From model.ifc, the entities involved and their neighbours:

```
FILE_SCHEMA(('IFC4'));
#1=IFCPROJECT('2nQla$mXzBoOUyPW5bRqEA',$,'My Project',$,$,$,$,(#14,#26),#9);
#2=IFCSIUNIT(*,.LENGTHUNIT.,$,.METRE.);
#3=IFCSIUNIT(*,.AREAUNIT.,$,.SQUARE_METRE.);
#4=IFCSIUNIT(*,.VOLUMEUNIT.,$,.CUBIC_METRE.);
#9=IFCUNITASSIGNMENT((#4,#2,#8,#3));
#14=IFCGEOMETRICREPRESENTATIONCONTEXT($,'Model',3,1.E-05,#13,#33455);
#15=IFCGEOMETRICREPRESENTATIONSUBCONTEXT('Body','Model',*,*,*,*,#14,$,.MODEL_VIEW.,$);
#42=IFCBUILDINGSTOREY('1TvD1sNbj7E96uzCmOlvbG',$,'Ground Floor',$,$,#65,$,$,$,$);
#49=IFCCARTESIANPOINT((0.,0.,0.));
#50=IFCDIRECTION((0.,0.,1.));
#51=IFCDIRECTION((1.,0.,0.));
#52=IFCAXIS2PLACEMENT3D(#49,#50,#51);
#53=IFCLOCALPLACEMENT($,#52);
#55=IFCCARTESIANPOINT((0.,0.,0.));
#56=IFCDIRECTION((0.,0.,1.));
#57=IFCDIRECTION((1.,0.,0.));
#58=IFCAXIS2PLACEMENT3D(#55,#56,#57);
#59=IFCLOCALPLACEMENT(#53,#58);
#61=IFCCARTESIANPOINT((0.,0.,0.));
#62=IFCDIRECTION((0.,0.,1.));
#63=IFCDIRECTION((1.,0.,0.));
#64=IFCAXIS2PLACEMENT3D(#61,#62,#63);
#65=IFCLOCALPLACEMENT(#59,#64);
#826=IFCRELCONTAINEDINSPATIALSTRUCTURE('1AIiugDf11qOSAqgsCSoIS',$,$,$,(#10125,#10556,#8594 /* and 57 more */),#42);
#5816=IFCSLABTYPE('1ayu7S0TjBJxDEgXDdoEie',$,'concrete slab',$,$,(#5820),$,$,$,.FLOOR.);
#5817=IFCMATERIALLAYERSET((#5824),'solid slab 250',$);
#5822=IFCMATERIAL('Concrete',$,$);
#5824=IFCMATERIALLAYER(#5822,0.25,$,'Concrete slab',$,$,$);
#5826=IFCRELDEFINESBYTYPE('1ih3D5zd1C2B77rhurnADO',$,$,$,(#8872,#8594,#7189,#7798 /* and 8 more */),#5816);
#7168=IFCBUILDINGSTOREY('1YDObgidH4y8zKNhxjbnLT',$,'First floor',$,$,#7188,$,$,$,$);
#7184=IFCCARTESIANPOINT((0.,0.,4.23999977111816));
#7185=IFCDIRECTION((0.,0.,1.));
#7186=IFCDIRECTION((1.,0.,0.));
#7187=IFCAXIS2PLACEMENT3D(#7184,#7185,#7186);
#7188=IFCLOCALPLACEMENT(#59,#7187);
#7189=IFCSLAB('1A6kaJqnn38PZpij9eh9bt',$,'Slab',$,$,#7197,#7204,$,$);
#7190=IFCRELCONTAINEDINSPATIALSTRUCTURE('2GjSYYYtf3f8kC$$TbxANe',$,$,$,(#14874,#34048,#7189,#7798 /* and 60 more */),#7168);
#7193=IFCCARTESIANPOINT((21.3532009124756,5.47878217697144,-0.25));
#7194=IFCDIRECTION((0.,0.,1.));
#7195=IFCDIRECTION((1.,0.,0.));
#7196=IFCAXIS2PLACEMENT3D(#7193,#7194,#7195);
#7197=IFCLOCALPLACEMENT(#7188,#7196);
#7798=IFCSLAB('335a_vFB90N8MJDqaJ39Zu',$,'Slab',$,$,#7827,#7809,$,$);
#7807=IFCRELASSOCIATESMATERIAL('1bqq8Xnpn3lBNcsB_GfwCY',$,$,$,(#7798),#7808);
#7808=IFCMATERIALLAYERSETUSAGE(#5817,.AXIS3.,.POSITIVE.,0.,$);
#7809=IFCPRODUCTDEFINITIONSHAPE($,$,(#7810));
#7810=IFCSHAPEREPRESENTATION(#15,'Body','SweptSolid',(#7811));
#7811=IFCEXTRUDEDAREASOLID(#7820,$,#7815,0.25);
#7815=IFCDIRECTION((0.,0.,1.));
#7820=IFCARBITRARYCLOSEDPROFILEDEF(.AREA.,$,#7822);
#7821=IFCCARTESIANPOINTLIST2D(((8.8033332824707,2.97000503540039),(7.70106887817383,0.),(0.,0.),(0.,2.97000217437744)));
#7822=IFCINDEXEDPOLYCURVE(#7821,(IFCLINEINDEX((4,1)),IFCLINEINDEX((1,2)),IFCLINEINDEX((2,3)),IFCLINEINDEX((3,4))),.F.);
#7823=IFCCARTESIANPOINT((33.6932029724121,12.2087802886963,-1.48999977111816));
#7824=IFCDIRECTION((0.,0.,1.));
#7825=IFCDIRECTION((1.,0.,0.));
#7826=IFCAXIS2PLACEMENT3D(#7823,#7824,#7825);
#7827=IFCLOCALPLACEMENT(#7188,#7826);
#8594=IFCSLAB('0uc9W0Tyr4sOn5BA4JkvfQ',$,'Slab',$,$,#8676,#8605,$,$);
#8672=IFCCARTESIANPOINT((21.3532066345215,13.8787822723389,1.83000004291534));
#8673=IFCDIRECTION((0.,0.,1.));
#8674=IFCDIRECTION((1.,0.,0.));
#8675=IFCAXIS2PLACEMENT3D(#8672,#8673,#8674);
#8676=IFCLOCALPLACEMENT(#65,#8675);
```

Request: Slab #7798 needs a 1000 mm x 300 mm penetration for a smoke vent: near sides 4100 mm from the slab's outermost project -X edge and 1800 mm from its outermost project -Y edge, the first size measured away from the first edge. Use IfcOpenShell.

```python
import numpy as np
import ifcopenshell
import ifcopenshell.api.feature
import ifcopenshell.api.geometry
import ifcopenshell.api.root
import ifcopenshell.geom
import ifcopenshell.util.placement
import ifcopenshell.util.representation
import ifcopenshell.util.shape
import ifcopenshell.util.unit

model = ifcopenshell.open("model.ifc")
unit_scale = ifcopenshell.util.unit.calculate_unit_scale(model)
settings = ifcopenshell.geom.settings()


def volume(element):
    """Net volume in cubic metres, openings subtracted."""
    shape = ifcopenshell.geom.create_shape(settings, element)
    return ifcopenshell.util.shape.get_volume(shape.geometry)


slab = model.by_id(7798)
before = volume(slab)

# Extent in the slab's own axes, in metres. The edges named are its -X and -Y sides.
slab_shape = ifcopenshell.geom.create_shape(settings, slab)
vertices = ifcopenshell.util.shape.get_vertices(slab_shape.geometry)
x_min, y_min, bottom = vertices.min(axis=0)
top = vertices[:, 2].max()

opening = ifcopenshell.api.root.create_entity(model, ifc_class="IfcOpeningElement", name="Smoke vent opening", predefined_type="OPENING")
context = ifcopenshell.util.representation.get_context(model, "Model", "Body", "MODEL_VIEW")
width, depth = 1, 0.3
outline = [(0.0, 0.0), (width, 0.0), (width, depth), (0.0, depth), (0.0, 0.0)]
# Overshoot both faces by 50 mm so the cut is clean.
shape = ifcopenshell.api.geometry.add_slab_representation(
    model, context=context, depth=top - bottom + 0.1, polyline=outline
)
ifcopenshell.api.geometry.assign_representation(model, product=opening, representation=shape)

matrix = ifcopenshell.util.placement.get_local_placement(slab.ObjectPlacement)
matrix[:, 3] = matrix @ np.append(np.array([x_min + 4.1, y_min + 1.8, bottom - 0.05]) / unit_scale, 1.0)
ifcopenshell.api.geometry.edit_object_placement(model, product=opening, matrix=matrix, is_si=False)
ifcopenshell.api.feature.add_feature(model, feature=opening, element=slab)

after = volume(slab)

print(f"slab volume {before:.3f} -> {after:.3f} m3")

model.write("model_rev.ifc")
```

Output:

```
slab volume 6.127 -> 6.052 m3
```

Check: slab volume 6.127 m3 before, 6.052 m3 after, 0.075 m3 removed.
